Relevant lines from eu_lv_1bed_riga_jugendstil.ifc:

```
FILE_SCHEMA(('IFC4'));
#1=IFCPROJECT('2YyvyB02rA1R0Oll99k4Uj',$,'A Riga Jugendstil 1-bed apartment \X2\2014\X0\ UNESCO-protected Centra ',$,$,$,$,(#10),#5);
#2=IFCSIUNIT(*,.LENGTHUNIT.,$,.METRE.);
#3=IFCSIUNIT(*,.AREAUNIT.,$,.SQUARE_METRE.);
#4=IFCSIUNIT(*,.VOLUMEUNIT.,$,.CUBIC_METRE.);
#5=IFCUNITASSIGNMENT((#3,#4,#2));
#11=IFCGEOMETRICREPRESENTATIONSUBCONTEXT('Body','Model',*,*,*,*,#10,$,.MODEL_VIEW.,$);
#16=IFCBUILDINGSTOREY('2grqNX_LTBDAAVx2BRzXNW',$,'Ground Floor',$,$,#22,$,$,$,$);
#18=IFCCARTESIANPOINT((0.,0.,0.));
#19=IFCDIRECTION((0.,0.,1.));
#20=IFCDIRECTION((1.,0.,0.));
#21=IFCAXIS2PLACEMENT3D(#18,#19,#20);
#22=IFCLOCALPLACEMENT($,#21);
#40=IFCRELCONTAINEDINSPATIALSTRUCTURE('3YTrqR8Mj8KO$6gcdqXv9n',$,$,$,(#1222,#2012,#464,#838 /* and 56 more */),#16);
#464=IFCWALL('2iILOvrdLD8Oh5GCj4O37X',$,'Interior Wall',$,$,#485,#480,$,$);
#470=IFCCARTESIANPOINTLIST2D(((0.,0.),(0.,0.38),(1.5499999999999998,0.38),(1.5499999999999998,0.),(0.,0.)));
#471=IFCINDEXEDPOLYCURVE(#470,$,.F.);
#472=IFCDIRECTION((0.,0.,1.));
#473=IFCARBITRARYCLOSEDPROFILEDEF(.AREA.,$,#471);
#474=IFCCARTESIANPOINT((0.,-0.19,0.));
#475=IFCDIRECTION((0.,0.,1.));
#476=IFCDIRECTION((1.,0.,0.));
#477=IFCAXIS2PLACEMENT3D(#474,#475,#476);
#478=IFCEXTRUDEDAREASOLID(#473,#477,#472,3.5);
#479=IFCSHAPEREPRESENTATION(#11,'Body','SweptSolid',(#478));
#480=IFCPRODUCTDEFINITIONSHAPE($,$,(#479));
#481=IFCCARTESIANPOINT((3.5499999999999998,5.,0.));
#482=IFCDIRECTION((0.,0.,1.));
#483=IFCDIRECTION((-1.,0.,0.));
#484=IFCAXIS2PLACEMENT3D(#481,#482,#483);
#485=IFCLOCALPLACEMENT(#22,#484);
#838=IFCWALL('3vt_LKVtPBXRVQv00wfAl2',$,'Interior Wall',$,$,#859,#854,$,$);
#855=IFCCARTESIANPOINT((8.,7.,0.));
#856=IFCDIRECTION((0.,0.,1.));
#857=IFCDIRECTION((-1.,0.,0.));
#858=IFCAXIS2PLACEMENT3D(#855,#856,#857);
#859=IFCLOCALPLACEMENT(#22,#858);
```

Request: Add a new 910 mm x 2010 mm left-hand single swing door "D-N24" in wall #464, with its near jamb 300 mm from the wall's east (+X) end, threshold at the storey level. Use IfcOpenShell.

```python
import numpy as np
import ifcopenshell
import ifcopenshell.api.feature
import ifcopenshell.api.geometry
import ifcopenshell.api.root
import ifcopenshell.api.spatial
import ifcopenshell.geom
import ifcopenshell.util.element
import ifcopenshell.util.placement
import ifcopenshell.util.representation
import ifcopenshell.util.shape
import ifcopenshell.util.unit

model = ifcopenshell.open("eu_lv_1bed_riga_jugendstil.ifc")
unit_scale = ifcopenshell.util.unit.calculate_unit_scale(model)
settings = ifcopenshell.geom.settings()


def volume(element):
    """Net volume in cubic metres, openings subtracted."""
    shape = ifcopenshell.geom.create_shape(settings, element)
    return ifcopenshell.util.shape.get_volume(shape.geometry)


wall = model.by_guid("2iILOvrdLD8Oh5GCj4O37X")
storey = ifcopenshell.util.element.get_container(wall, ifc_class="IfcBuildingStorey")
context = ifcopenshell.util.representation.get_context(model, "Model", "Body", "MODEL_VIEW")
before = volume(wall)

width, height, from_end, sill = 0.91, 2.01, 0.3, 0.0  # metres

# The wall runs along its own X axis, and the end named is its -X end.
wall_shape = ifcopenshell.geom.create_shape(settings, wall)
x, y, z = ifcopenshell.util.shape.get_vertices(wall_shape.geometry).T
start = x.min() + from_end
face, thickness = float(y.min()), float(y.max() - y.min())
wall_matrix = ifcopenshell.util.placement.get_local_placement(wall.ObjectPlacement)
level = ifcopenshell.util.placement.get_local_placement(storey.ObjectPlacement)[2, 3]


def in_wall(x, y):
    """Placement at x, y metres in the wall's axes, at sill height."""
    matrix = wall_matrix.copy()
    matrix[:, 3] = wall_matrix @ np.array([x / unit_scale, y / unit_scale, 0.0, 1.0])
    matrix[2, 3] = level + sill / unit_scale
    return matrix


# Opening: a box that overshoots both wall faces by 50 mm.
opening = ifcopenshell.api.root.create_entity(model, ifc_class="IfcOpeningElement", predefined_type="OPENING")
box = ifcopenshell.api.geometry.add_wall_representation(
    model, context=context, length=width, height=height, thickness=thickness + 0.1
)
ifcopenshell.api.geometry.assign_representation(model, product=opening, representation=box)
ifcopenshell.api.geometry.edit_object_placement(model, product=opening, matrix=in_wall(start, face - 0.05), is_si=False)
ifcopenshell.api.feature.add_feature(model, feature=opening, element=wall)

door = ifcopenshell.api.root.create_entity(model, ifc_class="IfcDoor", name="D-N24", predefined_type="DOOR")
door.OverallWidth, door.OverallHeight = width / unit_scale, height / unit_scale
door.OperationType = "SINGLE_SWING_LEFT"
body = ifcopenshell.api.geometry.add_door_representation(
    model,
    context=context,
    overall_width=door.OverallWidth,
    overall_height=door.OverallHeight,
    operation_type="SINGLE_SWING_LEFT",
    lining_properties={"LiningDepth": thickness / unit_scale, "ThresholdDepth": thickness / unit_scale},
)
ifcopenshell.api.geometry.assign_representation(model, product=door, representation=body)
ifcopenshell.api.spatial.assign_container(model, products=[door], relating_structure=storey)
ifcopenshell.api.feature.add_filling(model, opening=opening, element=door)

# The lining spans the wall, so the door starts at the wall face.
ifcopenshell.api.geometry.edit_object_placement(model, product=door, matrix=in_wall(start, face), is_si=False)

after = volume(wall)

print(f"wall volume {before:.3f} -> {after:.3f} m3")

model.write("eu_lv_1bed_riga_jugendstil-out.ifc")
```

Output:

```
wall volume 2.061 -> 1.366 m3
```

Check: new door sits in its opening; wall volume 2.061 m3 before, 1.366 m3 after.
